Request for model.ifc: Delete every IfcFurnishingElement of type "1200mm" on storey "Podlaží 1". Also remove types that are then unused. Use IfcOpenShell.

First a look at what the model holds.

```python
import ifcopenshell
import ifcopenshell.util.element

model = ifcopenshell.open("model.ifc")
print(model.schema)
storey = next(s for s in model.by_type("IfcBuildingStorey") if s.Name == "Podlaží 1")
furniture = [e for e in ifcopenshell.util.element.get_decomposition(storey) if e.is_a("IfcFurnishingElement")]
seen = {}
for e in furniture:
    element_type = ifcopenshell.util.element.get_type(e)
    name = element_type.Name if element_type not in (None, e) else None
    seen[name] = seen.get(name, 0) + 1
for name, count in sorted(seen.items(), key=str):
    print(count, "x", name)
```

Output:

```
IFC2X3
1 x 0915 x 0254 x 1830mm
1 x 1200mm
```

```python
import ifcopenshell
import ifcopenshell.api.root
import ifcopenshell.util.element

model = ifcopenshell.open("model.ifc")

storey = next(s for s in model.by_type("IfcBuildingStorey") if s.Name == "Podlaží 1")
furniture = [e for e in ifcopenshell.util.element.get_decomposition(storey) if e.is_a("IfcFurnishingElement")]
targets = [e for e in furniture if (t := ifcopenshell.util.element.get_type(e)) not in (None, e) and t.Name == "1200mm"]
types = {ifcopenshell.util.element.get_type(e) for e in targets} - {None, *targets}

for e in targets:
    ifcopenshell.api.root.remove_product(model, product=e)
print(len(targets), "removed")

unused = [t for t in types if not ifcopenshell.util.element.get_types(t)]
for t in unused:
    ifcopenshell.api.root.remove_product(model, product=t)
print(len(unused), "unused types removed")

model.write("model_rev.ifc")
```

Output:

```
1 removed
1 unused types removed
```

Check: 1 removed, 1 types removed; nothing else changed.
